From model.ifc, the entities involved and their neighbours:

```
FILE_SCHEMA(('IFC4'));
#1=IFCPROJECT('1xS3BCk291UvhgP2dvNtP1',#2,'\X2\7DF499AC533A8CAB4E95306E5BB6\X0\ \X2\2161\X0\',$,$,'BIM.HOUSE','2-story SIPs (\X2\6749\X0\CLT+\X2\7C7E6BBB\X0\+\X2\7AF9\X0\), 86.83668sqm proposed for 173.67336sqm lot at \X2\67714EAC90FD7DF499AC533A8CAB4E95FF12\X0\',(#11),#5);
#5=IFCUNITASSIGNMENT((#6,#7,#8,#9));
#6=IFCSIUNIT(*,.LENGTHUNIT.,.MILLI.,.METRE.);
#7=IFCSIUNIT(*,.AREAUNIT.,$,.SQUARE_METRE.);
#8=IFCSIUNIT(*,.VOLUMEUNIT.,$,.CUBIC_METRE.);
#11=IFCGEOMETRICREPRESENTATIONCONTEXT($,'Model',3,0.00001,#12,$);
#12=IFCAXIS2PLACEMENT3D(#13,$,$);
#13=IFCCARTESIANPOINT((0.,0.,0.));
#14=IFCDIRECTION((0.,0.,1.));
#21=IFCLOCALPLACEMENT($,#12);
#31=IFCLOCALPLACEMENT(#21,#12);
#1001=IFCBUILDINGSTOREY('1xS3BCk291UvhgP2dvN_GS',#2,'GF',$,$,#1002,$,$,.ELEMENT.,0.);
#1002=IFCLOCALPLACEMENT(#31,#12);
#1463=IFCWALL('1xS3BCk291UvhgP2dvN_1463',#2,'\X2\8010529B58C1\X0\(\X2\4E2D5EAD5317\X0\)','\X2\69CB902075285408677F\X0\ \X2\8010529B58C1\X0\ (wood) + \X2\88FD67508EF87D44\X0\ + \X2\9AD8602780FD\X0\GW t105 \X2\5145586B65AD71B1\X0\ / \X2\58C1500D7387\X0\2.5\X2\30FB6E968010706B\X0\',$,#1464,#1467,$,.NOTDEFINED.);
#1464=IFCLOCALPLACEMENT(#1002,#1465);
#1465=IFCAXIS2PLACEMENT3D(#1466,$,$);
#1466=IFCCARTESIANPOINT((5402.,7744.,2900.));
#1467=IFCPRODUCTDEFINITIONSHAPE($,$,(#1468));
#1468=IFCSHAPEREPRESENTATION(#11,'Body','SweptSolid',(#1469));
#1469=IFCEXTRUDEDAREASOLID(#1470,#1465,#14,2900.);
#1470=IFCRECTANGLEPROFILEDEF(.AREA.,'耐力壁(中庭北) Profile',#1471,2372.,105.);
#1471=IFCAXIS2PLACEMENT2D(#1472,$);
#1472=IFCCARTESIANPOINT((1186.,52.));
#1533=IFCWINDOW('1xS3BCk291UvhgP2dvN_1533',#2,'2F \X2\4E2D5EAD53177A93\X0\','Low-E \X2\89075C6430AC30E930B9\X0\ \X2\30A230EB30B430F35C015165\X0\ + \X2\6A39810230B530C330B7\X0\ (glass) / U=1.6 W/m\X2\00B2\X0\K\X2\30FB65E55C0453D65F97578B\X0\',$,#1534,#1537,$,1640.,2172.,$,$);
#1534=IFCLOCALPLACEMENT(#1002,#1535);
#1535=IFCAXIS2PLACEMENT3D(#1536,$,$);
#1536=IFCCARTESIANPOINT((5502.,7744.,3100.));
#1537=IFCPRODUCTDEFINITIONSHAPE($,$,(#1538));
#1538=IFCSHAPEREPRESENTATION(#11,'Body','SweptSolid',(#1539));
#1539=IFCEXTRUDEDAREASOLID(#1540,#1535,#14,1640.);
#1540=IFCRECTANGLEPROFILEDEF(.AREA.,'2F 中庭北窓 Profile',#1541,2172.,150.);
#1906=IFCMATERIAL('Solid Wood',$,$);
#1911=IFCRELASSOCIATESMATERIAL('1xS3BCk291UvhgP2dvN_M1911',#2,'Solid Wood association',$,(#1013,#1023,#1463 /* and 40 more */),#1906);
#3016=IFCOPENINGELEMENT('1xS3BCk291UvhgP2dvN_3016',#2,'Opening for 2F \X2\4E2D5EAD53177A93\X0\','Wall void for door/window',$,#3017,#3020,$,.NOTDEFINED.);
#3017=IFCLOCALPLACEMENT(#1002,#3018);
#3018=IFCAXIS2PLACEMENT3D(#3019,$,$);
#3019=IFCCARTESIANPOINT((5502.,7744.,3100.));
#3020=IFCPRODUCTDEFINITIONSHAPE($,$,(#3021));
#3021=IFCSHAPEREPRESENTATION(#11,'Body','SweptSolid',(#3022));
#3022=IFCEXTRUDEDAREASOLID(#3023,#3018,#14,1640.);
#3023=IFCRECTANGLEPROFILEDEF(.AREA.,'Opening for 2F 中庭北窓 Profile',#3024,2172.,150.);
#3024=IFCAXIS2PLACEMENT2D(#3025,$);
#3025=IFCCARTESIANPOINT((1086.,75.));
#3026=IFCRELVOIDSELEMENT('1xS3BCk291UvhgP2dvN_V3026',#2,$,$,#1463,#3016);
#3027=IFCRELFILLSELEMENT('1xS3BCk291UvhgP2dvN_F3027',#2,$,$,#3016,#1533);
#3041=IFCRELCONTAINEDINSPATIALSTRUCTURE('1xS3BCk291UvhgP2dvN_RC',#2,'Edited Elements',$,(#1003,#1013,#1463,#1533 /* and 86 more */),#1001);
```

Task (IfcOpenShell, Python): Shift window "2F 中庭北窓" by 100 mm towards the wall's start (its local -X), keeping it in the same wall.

```python
import ifcopenshell
import ifcopenshell.api.geometry
import ifcopenshell.util.placement

model = ifcopenshell.open("model.ifc")

window = model.by_guid("1xS3BCk291UvhgP2dvN_1533")
opening = window.FillsVoids[0].RelatingOpeningElement
wall = opening.VoidsElements[0].RelatingBuildingElement

wall_matrix = ifcopenshell.util.placement.get_local_placement(wall.ObjectPlacement)
shift = wall_matrix[:3, 0] * -100.0
before = ifcopenshell.util.placement.get_local_placement(window.ObjectPlacement)[:3, 3].copy()

# The window is not placed relative to its opening, so move both.
for product in (opening, window):
    matrix = ifcopenshell.util.placement.get_local_placement(product.ObjectPlacement)
    matrix[:3, 3] += shift
    ifcopenshell.api.geometry.edit_object_placement(model, product=product, matrix=matrix, is_si=False)

after = ifcopenshell.util.placement.get_local_placement(window.ObjectPlacement)[:3, 3]
print("window moved by", (after - before).round(3) + 0.0)

model.write("model_rev.ifc")
```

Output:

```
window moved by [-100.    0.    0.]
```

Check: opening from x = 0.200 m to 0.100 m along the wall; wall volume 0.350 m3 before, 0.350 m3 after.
